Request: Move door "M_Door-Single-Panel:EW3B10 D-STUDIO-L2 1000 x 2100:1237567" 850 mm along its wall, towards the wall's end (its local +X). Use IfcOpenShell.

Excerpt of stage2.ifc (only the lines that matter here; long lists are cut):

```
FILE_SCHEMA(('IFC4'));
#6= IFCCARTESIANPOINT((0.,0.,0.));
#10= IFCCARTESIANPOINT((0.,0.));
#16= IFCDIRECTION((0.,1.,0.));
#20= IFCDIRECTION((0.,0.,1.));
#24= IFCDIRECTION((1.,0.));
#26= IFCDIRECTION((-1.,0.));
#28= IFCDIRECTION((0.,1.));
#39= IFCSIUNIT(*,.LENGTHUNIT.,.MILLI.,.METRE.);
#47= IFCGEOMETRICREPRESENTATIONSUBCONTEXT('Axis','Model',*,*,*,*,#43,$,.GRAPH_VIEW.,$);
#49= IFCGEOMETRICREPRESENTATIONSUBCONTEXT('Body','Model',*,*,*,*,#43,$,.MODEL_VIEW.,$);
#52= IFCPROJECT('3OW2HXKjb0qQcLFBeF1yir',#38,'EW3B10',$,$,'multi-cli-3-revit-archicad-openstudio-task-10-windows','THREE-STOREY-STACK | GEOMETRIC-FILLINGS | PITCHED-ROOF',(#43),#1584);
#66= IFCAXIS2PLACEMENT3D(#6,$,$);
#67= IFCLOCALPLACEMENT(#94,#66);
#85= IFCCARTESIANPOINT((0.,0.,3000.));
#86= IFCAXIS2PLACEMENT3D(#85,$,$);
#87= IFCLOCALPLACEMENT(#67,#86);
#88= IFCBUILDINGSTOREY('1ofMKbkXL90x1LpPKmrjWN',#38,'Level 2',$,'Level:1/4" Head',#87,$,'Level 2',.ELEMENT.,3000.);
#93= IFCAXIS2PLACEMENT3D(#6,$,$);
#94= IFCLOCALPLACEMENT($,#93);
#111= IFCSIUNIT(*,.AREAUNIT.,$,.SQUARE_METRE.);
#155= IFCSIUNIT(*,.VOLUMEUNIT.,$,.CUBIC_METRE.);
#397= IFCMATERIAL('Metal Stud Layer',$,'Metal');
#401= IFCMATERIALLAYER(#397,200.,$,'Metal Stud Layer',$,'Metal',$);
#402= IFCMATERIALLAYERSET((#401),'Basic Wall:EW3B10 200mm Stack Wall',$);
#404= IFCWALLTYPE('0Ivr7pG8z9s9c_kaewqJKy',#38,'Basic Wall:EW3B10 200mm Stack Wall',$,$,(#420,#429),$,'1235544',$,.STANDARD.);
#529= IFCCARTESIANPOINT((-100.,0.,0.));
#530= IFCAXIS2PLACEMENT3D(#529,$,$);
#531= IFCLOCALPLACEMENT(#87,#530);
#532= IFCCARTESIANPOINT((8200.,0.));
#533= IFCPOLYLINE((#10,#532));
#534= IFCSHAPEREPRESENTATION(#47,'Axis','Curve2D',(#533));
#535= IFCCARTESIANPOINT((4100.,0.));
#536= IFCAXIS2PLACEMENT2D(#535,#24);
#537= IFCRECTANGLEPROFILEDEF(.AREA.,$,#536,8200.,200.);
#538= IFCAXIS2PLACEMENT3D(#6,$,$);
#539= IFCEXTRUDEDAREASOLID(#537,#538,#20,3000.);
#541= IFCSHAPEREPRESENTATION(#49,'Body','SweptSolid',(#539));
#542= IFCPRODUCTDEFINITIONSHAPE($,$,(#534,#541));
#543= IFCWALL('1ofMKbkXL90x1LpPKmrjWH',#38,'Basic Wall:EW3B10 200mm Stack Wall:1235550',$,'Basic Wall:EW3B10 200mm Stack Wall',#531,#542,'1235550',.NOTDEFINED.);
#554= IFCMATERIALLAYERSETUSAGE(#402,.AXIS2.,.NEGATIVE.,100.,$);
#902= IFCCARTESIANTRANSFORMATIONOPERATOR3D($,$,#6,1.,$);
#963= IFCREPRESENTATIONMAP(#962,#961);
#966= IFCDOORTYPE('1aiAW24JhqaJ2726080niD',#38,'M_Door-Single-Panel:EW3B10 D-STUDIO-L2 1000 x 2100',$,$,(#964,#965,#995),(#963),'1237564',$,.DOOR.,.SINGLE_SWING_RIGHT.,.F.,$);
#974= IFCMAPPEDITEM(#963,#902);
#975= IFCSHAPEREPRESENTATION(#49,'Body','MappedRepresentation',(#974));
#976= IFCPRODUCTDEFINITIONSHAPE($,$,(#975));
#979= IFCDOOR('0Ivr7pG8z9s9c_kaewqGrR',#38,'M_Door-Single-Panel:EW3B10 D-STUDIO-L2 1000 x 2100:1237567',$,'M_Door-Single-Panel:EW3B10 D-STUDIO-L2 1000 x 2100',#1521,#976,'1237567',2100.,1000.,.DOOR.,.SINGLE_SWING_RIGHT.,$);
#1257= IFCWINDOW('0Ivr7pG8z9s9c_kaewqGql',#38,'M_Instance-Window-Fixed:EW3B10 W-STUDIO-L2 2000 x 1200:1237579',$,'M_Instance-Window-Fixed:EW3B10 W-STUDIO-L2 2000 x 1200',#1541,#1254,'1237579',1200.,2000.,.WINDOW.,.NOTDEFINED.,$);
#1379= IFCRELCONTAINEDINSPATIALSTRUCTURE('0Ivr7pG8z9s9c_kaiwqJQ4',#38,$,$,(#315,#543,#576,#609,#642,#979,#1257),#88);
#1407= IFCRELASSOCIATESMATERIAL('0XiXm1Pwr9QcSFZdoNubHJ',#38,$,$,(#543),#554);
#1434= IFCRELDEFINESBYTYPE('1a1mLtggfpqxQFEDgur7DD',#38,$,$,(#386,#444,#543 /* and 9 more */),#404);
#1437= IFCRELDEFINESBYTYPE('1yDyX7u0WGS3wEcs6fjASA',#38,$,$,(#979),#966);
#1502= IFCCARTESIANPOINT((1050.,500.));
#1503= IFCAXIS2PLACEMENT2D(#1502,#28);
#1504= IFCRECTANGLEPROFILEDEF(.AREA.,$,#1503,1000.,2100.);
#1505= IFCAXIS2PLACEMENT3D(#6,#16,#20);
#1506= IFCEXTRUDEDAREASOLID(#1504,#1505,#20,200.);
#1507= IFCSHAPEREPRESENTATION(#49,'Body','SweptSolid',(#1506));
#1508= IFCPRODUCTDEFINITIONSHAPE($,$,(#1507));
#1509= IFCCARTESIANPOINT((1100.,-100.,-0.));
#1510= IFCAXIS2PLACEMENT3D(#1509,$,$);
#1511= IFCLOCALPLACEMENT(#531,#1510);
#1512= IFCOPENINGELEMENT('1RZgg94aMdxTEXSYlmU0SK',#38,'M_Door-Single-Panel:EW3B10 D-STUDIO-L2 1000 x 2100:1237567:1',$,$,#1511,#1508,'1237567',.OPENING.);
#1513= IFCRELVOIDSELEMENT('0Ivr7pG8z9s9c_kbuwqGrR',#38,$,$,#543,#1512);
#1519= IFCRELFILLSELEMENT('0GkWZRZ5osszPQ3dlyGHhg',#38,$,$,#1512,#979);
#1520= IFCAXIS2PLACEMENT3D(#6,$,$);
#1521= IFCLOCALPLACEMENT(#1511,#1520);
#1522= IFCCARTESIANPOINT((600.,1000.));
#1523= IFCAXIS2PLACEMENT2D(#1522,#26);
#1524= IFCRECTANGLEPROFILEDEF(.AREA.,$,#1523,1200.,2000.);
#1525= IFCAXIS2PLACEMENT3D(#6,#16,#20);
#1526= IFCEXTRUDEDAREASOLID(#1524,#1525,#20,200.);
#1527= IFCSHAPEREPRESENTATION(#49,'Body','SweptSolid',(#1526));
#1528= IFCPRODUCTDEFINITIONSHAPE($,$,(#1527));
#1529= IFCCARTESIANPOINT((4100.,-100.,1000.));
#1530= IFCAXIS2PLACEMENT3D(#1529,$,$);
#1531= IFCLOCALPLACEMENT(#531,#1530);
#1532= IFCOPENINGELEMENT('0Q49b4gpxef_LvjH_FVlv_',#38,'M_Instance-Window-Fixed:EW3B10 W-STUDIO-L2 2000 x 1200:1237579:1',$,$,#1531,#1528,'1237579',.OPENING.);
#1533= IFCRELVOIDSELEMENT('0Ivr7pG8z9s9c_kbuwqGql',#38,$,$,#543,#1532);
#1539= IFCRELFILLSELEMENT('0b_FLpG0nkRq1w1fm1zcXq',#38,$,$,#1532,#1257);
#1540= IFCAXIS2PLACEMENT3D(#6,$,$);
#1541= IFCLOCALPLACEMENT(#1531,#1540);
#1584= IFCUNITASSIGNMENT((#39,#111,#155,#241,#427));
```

```python
import ifcopenshell
import ifcopenshell.api.geometry
import ifcopenshell.util.placement

model = ifcopenshell.open("stage2.ifc")

door = model.by_guid("0Ivr7pG8z9s9c_kaewqGrR")
opening = door.FillsVoids[0].RelatingOpeningElement
wall = opening.VoidsElements[0].RelatingBuildingElement

wall_matrix = ifcopenshell.util.placement.get_local_placement(wall.ObjectPlacement)
shift = wall_matrix[:3, 0] * 850.0
before = ifcopenshell.util.placement.get_local_placement(door.ObjectPlacement)[:3, 3].copy()

# The door is placed relative to its opening, so it follows when the opening moves.
matrix = ifcopenshell.util.placement.get_local_placement(opening.ObjectPlacement)
matrix[:3, 3] += shift
ifcopenshell.api.geometry.edit_object_placement(
    model, product=opening, matrix=matrix, is_si=False, should_transform_children=True
)

after = ifcopenshell.util.placement.get_local_placement(door.ObjectPlacement)[:3, 3]
print("door moved by", (after - before).round(3) + 0.0)

model.write("stage2_v2.ifc")
```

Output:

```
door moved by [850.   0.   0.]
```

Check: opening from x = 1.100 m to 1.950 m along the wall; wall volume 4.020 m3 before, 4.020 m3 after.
